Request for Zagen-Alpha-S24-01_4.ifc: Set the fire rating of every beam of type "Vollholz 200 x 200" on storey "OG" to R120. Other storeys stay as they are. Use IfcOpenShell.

First a look at what the model holds.

```python
import ifcopenshell
import ifcopenshell.util.element

model = ifcopenshell.open("Zagen-Alpha-S24-01_4.ifc")
print(model.schema)
storey = next(s for s in model.by_type("IfcBuildingStorey") if s.Name == "OG")
beams = [e for e in ifcopenshell.util.element.get_decomposition(storey) if e.is_a("IfcBeam")]
seen = {}
for e in beams:
    element_type = ifcopenshell.util.element.get_type(e)
    key = (element_type.Name if element_type != e and element_type else None, ifcopenshell.util.element.get_pset(e, "Pset_BeamCommon", "FireRating"))
    seen[key] = seen.get(key, 0) + 1
for (name, value), count in sorted(seen.items(), key=str):
    print(count, "x", name, "|", value)
```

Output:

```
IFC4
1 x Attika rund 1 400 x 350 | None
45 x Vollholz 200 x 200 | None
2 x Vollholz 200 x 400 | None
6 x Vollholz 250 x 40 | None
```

```python
import ifcopenshell
import ifcopenshell.api.pset
import ifcopenshell.util.element

model = ifcopenshell.open("Zagen-Alpha-S24-01_4.ifc")

storey = next(s for s in model.by_type("IfcBuildingStorey") if s.Name == "OG")
beams = [e for e in ifcopenshell.util.element.get_decomposition(storey) if e.is_a("IfcBeam")]

count = 0
for e in beams:
    element_type = ifcopenshell.util.element.get_type(e)
    if element_type in (None, e) or element_type.Name != "Vollholz 200 x 200":
        continue
    # add_pset returns the element's existing set when there is one.
    pset = ifcopenshell.api.pset.add_pset(model, product=e, name="Pset_BeamCommon")
    ifcopenshell.api.pset.edit_pset(model, pset=pset, properties={"FireRating": "R120"})
    count += 1

print(count, "beams updated")

model.write("Zagen-Alpha-S24-01_4-out.ifc")
```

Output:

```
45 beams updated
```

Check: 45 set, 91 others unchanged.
